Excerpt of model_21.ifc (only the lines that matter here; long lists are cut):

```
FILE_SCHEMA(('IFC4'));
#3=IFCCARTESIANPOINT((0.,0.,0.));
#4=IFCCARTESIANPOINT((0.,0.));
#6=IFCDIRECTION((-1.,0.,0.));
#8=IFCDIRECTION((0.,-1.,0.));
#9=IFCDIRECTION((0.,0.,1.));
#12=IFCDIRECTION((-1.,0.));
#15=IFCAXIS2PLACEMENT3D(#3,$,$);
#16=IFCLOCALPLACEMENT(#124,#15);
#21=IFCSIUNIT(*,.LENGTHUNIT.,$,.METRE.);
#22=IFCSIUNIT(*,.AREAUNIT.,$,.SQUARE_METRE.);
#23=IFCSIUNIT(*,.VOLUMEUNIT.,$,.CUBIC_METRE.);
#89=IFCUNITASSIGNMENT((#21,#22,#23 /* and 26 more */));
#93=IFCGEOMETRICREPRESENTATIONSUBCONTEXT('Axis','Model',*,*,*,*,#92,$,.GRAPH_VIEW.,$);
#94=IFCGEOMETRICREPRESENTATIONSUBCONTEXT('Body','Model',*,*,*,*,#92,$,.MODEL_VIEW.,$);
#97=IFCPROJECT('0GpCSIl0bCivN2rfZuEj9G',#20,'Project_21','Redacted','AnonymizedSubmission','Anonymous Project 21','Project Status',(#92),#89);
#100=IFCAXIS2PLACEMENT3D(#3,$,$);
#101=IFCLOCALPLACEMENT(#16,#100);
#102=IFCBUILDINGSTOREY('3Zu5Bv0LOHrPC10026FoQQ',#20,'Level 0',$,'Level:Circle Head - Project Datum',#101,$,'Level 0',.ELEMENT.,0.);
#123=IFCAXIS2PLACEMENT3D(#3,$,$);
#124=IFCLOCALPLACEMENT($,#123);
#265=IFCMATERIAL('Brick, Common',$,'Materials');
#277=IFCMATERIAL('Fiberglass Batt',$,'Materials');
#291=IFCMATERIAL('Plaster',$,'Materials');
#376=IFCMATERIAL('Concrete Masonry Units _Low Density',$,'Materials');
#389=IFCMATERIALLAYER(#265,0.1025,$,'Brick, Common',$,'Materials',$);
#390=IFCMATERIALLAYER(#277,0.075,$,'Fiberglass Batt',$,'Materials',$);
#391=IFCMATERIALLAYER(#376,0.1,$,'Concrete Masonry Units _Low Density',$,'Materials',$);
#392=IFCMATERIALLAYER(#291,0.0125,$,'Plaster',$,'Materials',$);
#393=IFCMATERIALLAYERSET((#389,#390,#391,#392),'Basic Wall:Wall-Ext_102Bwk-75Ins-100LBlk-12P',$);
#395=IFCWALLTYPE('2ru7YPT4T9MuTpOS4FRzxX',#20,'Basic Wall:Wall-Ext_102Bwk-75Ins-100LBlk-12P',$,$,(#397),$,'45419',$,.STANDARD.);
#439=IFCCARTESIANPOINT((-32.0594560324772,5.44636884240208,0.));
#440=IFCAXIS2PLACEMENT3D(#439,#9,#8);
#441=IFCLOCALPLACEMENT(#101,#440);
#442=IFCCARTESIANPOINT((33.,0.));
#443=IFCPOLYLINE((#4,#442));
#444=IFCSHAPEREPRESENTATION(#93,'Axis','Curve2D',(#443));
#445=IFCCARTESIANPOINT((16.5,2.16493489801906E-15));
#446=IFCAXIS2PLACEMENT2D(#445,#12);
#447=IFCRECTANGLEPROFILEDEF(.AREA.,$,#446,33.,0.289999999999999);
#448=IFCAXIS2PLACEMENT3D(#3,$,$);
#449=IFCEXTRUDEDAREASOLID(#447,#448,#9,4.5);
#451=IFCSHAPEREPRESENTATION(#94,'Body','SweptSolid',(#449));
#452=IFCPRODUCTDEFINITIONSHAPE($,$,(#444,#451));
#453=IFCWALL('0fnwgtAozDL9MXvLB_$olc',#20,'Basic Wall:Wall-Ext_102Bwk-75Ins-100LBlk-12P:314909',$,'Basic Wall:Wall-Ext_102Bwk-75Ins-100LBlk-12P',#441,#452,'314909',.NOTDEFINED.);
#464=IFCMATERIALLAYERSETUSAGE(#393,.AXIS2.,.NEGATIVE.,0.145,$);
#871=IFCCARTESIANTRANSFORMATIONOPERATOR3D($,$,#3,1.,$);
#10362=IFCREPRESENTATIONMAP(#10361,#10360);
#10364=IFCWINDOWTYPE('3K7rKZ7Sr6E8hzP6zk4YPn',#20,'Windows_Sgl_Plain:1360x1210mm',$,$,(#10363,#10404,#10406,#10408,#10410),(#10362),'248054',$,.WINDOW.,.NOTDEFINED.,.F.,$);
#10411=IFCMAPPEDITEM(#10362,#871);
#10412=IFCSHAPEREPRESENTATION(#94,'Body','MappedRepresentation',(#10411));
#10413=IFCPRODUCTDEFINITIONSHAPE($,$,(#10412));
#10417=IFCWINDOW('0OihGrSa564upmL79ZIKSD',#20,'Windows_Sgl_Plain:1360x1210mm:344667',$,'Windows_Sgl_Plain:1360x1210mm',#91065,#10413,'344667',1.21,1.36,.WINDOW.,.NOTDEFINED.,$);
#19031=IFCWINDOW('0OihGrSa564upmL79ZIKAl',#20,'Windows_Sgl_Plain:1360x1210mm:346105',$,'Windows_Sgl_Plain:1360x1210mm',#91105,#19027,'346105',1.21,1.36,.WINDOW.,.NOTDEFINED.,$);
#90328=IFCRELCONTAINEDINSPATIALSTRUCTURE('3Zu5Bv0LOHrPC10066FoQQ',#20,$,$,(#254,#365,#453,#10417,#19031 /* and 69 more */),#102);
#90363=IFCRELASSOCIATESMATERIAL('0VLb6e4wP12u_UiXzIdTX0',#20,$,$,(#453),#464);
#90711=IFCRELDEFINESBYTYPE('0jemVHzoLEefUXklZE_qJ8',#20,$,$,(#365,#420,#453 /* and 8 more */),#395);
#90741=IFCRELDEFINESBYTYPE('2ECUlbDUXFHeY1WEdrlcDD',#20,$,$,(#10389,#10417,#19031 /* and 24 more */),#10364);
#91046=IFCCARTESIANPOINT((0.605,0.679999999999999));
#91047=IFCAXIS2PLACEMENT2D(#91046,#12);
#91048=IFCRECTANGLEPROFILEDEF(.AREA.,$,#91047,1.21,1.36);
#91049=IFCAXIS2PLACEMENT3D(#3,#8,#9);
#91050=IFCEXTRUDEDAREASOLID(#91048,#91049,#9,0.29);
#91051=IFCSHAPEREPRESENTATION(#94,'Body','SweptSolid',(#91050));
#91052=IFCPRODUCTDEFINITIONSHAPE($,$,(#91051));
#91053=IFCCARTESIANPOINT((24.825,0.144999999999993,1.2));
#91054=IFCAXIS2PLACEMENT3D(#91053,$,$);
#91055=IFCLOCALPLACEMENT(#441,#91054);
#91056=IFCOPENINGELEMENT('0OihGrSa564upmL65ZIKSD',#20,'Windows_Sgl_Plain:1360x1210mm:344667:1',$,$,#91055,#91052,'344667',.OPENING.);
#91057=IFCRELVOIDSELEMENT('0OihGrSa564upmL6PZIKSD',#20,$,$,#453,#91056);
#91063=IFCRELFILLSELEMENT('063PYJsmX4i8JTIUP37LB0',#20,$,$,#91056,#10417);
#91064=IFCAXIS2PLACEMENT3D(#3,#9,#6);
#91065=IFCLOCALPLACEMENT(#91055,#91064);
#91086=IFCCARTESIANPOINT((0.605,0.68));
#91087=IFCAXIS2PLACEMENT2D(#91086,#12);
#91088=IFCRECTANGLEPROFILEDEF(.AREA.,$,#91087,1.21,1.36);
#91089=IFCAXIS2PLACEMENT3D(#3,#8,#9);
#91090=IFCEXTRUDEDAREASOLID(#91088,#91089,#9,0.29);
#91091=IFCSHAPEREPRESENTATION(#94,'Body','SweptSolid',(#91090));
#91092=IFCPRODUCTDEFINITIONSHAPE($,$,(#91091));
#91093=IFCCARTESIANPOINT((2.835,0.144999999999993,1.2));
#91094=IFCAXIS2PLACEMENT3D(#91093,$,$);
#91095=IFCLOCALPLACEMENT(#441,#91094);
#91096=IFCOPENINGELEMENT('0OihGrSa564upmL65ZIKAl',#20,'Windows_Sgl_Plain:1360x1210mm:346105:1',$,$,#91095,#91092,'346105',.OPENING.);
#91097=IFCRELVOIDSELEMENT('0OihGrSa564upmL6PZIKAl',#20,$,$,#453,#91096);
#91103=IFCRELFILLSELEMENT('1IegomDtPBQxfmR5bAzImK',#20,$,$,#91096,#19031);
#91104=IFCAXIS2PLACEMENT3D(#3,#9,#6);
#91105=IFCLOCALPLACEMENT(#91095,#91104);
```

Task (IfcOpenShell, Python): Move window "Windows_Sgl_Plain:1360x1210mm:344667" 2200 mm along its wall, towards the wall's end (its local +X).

```python
import ifcopenshell
import ifcopenshell.api.geometry
import ifcopenshell.util.placement
import ifcopenshell.util.unit

model = ifcopenshell.open("model_21.ifc")
unit_scale = ifcopenshell.util.unit.calculate_unit_scale(model)

window = model.by_id(10417)
opening = window.FillsVoids[0].RelatingOpeningElement
wall = opening.VoidsElements[0].RelatingBuildingElement

wall_matrix = ifcopenshell.util.placement.get_local_placement(wall.ObjectPlacement)
shift = wall_matrix[:3, 0] * 2.2 / unit_scale
before = ifcopenshell.util.placement.get_local_placement(window.ObjectPlacement)[:3, 3].copy()

# The window is placed relative to its opening, so it follows when the opening moves.
matrix = ifcopenshell.util.placement.get_local_placement(opening.ObjectPlacement)
matrix[:3, 3] += shift
ifcopenshell.api.geometry.edit_object_placement(
    model, product=opening, matrix=matrix, is_si=False, should_transform_children=True
)

after = ifcopenshell.util.placement.get_local_placement(window.ObjectPlacement)[:3, 3]
print("window moved by", (after - before).round(3) + 0.0)

model.write("model_21_edited.ifc")
```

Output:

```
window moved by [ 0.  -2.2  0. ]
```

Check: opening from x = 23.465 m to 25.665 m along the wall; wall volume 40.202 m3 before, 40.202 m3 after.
